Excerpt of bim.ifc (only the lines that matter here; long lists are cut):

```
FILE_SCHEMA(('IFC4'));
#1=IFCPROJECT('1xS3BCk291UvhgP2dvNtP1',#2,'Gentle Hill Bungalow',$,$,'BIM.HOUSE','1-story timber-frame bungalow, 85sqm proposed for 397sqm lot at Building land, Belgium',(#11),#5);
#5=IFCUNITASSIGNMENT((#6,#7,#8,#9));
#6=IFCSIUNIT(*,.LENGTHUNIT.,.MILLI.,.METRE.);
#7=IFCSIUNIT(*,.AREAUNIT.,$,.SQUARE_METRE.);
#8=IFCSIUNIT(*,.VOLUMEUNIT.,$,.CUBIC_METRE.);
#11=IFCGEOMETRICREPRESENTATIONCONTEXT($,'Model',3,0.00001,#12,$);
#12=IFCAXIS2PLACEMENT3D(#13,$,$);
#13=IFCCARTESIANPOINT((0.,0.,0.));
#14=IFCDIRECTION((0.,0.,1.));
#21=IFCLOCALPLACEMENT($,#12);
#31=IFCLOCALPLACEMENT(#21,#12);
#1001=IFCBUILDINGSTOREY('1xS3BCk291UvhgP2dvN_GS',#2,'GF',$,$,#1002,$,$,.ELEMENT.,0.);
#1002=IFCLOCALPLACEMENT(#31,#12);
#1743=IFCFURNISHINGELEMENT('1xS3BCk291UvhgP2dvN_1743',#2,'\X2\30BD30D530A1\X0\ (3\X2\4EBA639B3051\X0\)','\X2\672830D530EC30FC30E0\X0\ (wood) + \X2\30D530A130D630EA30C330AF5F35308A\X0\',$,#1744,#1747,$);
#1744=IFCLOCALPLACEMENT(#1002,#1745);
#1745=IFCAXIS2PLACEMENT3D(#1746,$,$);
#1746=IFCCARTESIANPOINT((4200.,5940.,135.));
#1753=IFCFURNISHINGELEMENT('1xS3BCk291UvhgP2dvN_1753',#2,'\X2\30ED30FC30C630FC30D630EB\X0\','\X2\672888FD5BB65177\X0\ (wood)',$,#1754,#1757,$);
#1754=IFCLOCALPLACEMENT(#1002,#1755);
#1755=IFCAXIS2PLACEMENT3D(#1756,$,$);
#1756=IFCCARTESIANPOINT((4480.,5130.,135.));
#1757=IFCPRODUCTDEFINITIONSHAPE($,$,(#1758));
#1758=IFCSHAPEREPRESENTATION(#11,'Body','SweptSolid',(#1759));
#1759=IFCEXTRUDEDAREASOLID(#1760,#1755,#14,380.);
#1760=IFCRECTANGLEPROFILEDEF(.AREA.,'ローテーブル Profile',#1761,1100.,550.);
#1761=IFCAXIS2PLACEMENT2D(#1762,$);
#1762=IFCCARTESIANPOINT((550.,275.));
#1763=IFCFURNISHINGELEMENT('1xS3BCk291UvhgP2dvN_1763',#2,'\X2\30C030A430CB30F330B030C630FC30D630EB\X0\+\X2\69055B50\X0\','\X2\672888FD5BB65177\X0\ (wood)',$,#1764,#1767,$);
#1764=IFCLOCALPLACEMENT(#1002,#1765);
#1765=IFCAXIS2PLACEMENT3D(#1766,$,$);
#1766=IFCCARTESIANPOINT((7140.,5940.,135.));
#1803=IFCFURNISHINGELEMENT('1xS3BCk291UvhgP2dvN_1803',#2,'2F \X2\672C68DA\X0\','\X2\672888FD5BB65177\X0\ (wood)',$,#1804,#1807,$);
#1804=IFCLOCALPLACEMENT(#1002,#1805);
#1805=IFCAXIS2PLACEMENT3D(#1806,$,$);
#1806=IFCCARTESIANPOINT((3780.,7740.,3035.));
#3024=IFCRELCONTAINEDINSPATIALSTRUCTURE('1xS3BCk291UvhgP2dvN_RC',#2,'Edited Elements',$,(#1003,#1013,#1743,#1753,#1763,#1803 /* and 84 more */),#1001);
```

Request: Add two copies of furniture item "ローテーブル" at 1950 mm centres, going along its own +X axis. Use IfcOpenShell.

```python
import ifcopenshell
import ifcopenshell.api.geometry
import ifcopenshell.api.root
import ifcopenshell.util.element
import ifcopenshell.util.placement
import ifcopenshell.util.unit

model = ifcopenshell.open("bim.ifc")
unit_scale = ifcopenshell.util.unit.calculate_unit_scale(model)


def reuse_history(source, copy):
    """copy_class also copies each property set's owner history, people and application; keep the originals."""
    for rel in copy.IsDefinedBy:
        if rel.is_a("IfcRelDefinesByProperties") and (history := rel.RelatingPropertyDefinition.OwnerHistory):
            rel.RelatingPropertyDefinition.OwnerHistory = source.OwnerHistory
            ifcopenshell.util.element.remove_deep2(model, history)


source = model.by_id(1753)
base = ifcopenshell.util.placement.get_local_placement(source.ObjectPlacement)
step = base[:3, 0] * 1.95 / unit_scale

for i in range(1, 3):
    copy = ifcopenshell.api.root.copy_class(model, product=source)
    copy.Representation = ifcopenshell.util.element.copy_deep(
        model, source.Representation, exclude=["IfcGeometricRepresentationContext", "IfcRepresentationMap"]
    )
    reuse_history(source, copy)
    matrix = base.copy()
    matrix[:3, 3] += i * step
    print("added at", matrix[:3, 3].round(3) + 0.0)
    ifcopenshell.api.geometry.edit_object_placement(model, product=copy, matrix=matrix, is_si=False)

model.write("bim_updated.ifc")
```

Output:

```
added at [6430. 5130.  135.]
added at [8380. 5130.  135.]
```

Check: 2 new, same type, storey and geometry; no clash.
